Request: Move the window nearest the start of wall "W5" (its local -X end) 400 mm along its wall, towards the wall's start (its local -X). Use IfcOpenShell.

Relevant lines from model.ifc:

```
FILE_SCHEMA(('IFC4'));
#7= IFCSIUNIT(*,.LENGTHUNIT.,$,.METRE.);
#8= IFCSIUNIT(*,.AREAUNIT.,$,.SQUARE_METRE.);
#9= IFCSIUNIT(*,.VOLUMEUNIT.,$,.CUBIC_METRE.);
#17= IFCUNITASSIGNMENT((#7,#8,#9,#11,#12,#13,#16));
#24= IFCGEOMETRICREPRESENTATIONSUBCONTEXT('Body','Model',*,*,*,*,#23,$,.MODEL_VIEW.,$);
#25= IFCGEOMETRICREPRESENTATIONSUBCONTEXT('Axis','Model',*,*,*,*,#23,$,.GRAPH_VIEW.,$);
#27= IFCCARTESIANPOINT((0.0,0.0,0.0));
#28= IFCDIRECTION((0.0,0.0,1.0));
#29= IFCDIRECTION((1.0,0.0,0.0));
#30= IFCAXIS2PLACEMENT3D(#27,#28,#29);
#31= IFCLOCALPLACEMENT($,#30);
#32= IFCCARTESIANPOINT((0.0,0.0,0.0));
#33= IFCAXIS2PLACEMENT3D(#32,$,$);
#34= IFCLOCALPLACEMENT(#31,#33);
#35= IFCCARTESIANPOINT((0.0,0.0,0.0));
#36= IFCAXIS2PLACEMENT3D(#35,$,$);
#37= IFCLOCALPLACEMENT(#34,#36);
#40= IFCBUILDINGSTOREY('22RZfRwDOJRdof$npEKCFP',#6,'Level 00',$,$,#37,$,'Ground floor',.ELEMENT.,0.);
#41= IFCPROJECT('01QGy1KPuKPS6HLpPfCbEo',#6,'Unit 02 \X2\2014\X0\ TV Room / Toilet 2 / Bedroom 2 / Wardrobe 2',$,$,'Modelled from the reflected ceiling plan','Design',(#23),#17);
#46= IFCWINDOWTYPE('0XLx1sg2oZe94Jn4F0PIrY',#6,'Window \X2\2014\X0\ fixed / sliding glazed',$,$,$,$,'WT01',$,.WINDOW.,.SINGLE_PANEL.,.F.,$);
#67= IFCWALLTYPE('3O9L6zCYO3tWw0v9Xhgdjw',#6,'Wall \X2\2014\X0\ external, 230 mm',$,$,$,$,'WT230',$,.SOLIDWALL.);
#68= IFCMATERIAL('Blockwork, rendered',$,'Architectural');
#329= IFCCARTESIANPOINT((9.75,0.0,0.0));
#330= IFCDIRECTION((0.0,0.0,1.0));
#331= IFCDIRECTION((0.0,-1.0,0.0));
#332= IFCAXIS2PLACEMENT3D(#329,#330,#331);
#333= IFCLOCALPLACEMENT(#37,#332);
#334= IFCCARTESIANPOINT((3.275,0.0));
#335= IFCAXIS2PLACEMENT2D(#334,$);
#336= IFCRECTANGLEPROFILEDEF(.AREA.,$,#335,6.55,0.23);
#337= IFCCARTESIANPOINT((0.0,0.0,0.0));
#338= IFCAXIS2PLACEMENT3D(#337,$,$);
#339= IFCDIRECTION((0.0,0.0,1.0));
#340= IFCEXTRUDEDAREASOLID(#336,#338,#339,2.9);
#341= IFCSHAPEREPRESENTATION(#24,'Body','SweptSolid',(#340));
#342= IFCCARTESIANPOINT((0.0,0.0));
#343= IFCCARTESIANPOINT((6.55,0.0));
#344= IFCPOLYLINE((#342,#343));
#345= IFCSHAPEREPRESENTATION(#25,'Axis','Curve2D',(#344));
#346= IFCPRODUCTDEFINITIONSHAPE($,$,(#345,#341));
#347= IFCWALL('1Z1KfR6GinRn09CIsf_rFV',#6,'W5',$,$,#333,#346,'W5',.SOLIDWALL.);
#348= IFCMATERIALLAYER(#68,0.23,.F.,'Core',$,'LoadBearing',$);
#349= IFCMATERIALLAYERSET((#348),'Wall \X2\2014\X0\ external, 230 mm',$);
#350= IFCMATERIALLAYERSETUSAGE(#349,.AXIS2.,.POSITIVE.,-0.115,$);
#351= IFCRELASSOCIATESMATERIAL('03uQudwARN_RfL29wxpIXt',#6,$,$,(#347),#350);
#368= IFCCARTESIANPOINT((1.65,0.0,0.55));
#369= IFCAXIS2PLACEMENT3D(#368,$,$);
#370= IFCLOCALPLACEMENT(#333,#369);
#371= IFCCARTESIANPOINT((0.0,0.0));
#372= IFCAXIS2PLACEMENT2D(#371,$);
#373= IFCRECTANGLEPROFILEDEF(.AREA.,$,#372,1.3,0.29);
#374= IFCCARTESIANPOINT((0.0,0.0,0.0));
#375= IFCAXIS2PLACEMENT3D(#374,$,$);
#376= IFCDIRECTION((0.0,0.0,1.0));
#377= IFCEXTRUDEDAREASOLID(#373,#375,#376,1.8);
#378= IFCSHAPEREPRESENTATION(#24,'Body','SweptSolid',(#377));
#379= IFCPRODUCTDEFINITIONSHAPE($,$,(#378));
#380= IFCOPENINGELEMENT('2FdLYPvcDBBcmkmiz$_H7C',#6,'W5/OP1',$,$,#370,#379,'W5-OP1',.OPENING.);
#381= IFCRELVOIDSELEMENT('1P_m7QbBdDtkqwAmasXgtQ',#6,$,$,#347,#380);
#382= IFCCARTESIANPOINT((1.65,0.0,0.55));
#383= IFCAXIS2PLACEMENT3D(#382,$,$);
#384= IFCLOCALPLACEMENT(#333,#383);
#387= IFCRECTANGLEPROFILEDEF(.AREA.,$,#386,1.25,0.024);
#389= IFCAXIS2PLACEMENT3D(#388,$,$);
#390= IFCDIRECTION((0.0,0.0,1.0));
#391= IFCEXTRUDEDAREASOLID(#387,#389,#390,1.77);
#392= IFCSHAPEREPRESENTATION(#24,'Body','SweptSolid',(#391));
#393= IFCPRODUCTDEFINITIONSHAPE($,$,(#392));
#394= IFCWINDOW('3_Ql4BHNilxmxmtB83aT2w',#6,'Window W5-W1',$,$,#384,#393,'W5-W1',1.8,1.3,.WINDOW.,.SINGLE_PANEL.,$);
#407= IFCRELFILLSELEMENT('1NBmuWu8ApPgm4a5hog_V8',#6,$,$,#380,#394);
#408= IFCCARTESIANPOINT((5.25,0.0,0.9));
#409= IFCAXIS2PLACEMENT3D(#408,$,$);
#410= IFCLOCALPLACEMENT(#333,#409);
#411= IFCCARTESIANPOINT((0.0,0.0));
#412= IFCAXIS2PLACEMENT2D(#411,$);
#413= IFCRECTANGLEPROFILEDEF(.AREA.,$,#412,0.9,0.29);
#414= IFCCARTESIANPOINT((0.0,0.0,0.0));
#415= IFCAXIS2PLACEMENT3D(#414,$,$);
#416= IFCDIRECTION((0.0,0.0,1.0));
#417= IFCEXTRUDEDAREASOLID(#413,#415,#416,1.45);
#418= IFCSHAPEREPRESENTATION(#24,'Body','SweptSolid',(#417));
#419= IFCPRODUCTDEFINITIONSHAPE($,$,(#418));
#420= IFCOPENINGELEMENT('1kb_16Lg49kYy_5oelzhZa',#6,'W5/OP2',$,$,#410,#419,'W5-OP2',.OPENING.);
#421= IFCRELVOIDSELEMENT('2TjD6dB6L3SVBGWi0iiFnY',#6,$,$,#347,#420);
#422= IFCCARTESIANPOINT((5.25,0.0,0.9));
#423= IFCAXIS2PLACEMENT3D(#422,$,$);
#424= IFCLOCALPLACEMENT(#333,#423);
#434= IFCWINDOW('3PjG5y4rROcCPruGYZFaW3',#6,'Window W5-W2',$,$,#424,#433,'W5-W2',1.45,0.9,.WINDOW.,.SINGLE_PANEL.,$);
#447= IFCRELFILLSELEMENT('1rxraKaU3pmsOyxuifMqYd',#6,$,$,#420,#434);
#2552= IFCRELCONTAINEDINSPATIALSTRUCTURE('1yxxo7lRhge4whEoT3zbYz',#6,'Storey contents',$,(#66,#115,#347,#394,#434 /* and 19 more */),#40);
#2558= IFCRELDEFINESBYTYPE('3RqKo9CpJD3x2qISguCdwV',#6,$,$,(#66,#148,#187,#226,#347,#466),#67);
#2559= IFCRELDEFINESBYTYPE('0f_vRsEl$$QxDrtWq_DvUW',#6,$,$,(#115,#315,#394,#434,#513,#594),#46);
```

```python
import ifcopenshell
import ifcopenshell.api.geometry
import ifcopenshell.util.placement
import ifcopenshell.util.unit

model = ifcopenshell.open("model.ifc")
unit_scale = ifcopenshell.util.unit.calculate_unit_scale(model)

window = model.by_id(394)
opening = window.FillsVoids[0].RelatingOpeningElement
wall = opening.VoidsElements[0].RelatingBuildingElement

wall_matrix = ifcopenshell.util.placement.get_local_placement(wall.ObjectPlacement)
shift = wall_matrix[:3, 0] * -0.4 / unit_scale
before = ifcopenshell.util.placement.get_local_placement(window.ObjectPlacement)[:3, 3].copy()

# The window is not placed relative to its opening, so move both.
for product in (opening, window):
    matrix = ifcopenshell.util.placement.get_local_placement(product.ObjectPlacement)
    matrix[:3, 3] += shift
    ifcopenshell.api.geometry.edit_object_placement(model, product=product, matrix=matrix, is_si=False)

after = ifcopenshell.util.placement.get_local_placement(window.ObjectPlacement)[:3, 3]
print("window moved by", (after - before).round(3) + 0.0)

model.write("model_updated.ifc")
```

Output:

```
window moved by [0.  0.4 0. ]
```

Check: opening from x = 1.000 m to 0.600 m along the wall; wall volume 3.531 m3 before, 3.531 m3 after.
